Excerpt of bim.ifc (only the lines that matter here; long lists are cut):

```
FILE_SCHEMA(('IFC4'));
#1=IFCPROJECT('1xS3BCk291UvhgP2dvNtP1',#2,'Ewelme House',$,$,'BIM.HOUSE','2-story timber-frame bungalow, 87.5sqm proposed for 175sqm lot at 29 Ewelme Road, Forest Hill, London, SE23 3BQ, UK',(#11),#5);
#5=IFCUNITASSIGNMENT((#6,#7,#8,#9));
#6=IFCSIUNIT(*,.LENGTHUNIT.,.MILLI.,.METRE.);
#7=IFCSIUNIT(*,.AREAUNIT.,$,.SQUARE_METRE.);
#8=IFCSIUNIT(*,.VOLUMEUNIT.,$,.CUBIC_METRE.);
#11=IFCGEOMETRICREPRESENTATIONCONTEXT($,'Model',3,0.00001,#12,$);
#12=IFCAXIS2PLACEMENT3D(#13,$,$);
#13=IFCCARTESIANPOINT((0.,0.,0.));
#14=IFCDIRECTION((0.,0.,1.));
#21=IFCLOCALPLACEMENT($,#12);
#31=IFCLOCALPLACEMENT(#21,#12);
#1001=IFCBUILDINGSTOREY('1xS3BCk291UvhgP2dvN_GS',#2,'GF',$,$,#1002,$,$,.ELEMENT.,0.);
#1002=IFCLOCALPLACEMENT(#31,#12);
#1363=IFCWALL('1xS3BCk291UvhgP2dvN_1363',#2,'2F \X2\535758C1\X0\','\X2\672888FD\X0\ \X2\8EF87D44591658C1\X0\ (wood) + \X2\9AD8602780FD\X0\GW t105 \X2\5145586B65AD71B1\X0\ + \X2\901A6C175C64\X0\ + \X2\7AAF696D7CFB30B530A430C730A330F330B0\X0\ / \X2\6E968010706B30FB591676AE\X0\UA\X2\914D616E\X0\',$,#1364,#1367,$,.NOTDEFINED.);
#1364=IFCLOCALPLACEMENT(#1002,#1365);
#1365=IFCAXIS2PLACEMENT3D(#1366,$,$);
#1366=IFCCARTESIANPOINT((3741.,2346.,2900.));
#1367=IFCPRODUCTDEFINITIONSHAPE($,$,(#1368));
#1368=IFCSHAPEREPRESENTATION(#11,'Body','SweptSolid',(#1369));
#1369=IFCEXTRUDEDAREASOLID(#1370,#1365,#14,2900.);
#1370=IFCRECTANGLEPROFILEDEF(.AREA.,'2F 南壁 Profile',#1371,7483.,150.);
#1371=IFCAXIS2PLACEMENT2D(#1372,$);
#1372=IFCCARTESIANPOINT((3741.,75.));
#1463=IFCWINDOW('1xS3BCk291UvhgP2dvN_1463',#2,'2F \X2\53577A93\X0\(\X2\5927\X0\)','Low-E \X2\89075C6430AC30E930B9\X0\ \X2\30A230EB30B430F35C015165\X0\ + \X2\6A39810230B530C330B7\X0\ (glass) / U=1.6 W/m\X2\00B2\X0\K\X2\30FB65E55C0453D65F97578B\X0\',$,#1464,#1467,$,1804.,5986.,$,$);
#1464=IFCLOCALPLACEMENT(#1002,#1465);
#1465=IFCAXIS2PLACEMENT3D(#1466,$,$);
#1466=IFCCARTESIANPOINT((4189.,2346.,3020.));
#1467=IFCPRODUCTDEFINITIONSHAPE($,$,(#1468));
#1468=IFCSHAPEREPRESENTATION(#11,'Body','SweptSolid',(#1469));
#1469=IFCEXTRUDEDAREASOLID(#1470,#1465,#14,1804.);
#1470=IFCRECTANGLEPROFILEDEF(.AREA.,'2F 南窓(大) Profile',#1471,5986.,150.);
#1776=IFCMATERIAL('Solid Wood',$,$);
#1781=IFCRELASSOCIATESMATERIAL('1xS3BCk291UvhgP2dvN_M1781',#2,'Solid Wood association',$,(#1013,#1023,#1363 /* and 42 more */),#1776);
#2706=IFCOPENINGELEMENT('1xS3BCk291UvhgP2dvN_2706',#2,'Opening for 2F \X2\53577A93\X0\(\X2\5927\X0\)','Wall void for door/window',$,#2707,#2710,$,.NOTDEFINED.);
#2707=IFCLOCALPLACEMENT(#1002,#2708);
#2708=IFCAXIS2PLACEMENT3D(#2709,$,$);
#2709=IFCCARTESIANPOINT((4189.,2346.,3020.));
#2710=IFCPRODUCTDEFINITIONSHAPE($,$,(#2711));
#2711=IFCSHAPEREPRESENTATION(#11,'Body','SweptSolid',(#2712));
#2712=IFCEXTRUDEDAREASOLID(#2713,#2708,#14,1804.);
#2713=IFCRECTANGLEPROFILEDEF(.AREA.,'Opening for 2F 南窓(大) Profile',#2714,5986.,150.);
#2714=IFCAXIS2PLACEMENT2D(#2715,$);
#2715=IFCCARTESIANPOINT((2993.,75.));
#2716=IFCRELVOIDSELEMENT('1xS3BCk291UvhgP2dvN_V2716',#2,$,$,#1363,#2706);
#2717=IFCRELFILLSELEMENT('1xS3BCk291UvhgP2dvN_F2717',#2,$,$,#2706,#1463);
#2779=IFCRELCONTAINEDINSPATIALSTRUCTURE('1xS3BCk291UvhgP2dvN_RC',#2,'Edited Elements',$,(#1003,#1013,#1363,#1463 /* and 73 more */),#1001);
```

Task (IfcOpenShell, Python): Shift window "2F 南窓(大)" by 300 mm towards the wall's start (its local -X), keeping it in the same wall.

```python
import ifcopenshell
import ifcopenshell.api.geometry
import ifcopenshell.util.placement

model = ifcopenshell.open("bim.ifc")

window = model.by_id(1463)
opening = window.FillsVoids[0].RelatingOpeningElement
wall = opening.VoidsElements[0].RelatingBuildingElement

wall_matrix = ifcopenshell.util.placement.get_local_placement(wall.ObjectPlacement)
shift = wall_matrix[:3, 0] * -300.0
before = ifcopenshell.util.placement.get_local_placement(window.ObjectPlacement)[:3, 3].copy()

# The window is not placed relative to its opening, so move both.
for product in (opening, window):
    matrix = ifcopenshell.util.placement.get_local_placement(product.ObjectPlacement)
    matrix[:3, 3] += shift
    ifcopenshell.api.geometry.edit_object_placement(model, product=product, matrix=matrix, is_si=False)

after = ifcopenshell.util.placement.get_local_placement(window.ObjectPlacement)[:3, 3]
print("window moved by", (after - before).round(3) + 0.0)

model.write("bim_v2.ifc")
```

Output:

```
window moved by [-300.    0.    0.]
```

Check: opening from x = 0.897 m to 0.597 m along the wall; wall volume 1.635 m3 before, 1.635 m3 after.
